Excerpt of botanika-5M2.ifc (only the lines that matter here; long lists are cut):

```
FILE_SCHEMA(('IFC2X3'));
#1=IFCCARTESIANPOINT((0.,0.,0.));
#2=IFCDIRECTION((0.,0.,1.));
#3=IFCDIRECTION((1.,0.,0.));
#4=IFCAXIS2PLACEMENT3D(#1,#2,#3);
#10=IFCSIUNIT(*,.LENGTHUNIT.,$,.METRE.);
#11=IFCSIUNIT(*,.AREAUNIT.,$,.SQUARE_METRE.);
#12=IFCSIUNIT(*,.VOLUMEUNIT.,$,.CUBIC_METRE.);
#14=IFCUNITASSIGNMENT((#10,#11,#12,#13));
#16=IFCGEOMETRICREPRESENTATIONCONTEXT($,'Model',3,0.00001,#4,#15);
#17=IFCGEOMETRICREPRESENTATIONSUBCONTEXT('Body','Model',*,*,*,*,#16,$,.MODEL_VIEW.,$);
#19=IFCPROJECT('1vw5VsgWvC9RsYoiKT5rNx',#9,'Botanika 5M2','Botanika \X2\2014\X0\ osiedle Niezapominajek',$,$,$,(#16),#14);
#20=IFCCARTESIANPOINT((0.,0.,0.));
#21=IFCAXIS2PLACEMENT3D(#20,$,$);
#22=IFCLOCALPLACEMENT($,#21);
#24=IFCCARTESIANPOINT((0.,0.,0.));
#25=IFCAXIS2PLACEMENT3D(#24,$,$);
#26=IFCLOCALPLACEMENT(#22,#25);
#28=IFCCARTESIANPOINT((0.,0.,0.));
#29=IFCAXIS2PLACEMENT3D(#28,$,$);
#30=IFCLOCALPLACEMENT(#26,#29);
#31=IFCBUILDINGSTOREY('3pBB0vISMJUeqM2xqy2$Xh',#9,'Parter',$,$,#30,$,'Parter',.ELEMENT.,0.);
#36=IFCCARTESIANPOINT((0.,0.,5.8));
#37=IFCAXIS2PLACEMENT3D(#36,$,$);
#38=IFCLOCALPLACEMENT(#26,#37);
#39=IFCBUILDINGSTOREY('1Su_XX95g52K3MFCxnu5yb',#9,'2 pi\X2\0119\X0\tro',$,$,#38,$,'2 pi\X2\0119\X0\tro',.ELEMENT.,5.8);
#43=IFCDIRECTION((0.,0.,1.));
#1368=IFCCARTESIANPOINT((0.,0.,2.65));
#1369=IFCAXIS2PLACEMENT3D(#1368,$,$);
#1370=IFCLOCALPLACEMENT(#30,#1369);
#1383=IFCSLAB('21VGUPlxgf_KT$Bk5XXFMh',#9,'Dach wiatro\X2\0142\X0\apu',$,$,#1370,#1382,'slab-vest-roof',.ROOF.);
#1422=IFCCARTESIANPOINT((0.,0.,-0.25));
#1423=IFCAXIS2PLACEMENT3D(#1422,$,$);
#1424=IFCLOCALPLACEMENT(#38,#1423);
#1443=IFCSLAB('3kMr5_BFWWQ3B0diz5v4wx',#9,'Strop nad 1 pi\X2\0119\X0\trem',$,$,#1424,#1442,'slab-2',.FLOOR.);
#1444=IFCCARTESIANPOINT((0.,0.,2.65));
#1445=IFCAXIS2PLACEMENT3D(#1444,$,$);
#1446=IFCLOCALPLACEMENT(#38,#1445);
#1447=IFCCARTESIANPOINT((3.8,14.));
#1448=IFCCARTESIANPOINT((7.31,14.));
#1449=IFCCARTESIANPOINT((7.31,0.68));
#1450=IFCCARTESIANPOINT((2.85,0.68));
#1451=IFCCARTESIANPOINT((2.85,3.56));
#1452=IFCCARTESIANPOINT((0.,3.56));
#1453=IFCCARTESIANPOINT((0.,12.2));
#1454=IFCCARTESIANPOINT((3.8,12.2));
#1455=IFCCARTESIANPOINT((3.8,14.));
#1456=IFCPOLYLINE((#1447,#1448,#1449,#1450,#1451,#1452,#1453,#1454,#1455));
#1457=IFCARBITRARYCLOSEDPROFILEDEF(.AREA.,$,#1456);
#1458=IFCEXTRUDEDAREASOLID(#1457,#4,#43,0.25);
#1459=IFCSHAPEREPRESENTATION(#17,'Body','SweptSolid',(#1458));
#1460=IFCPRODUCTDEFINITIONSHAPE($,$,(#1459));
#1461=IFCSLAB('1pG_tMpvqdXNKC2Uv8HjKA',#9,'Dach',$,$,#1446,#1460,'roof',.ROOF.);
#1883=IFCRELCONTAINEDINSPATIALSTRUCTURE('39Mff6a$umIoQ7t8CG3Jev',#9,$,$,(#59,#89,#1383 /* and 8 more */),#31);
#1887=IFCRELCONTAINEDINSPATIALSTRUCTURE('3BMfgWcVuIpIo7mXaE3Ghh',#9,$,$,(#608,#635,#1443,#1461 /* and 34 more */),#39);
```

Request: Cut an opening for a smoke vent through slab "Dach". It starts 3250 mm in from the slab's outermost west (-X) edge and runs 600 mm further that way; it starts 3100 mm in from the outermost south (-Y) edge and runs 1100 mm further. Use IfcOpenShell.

```python
import numpy as np
import ifcopenshell
import ifcopenshell.api.feature
import ifcopenshell.api.geometry
import ifcopenshell.api.root
import ifcopenshell.geom
import ifcopenshell.util.placement
import ifcopenshell.util.representation
import ifcopenshell.util.shape
import ifcopenshell.util.unit

model = ifcopenshell.open("botanika-5M2.ifc")
unit_scale = ifcopenshell.util.unit.calculate_unit_scale(model)
settings = ifcopenshell.geom.settings()


def volume(element):
    """Net volume in cubic metres, openings subtracted."""
    shape = ifcopenshell.geom.create_shape(settings, element)
    return ifcopenshell.util.shape.get_volume(shape.geometry)


slab = model.by_guid("1pG_tMpvqdXNKC2Uv8HjKA")
before = volume(slab)

# Extent in the slab's own axes, in metres. The edges named are its -X and -Y sides.
slab_shape = ifcopenshell.geom.create_shape(settings, slab)
vertices = ifcopenshell.util.shape.get_vertices(slab_shape.geometry)
x_min, y_min, bottom = vertices.min(axis=0)
top = vertices[:, 2].max()

opening = ifcopenshell.api.root.create_entity(model, ifc_class="IfcOpeningElement", name="Smoke vent opening")
context = ifcopenshell.util.representation.get_context(model, "Model", "Body", "MODEL_VIEW")
width, depth = 0.6, 1.1
outline = [(0.0, 0.0), (width, 0.0), (width, depth), (0.0, depth), (0.0, 0.0)]
# Overshoot both faces by 50 mm so the cut is clean.
shape = ifcopenshell.api.geometry.add_slab_representation(
    model, context=context, depth=top - bottom + 0.1, polyline=outline
)
ifcopenshell.api.geometry.assign_representation(model, product=opening, representation=shape)

matrix = ifcopenshell.util.placement.get_local_placement(slab.ObjectPlacement)
matrix[:, 3] = matrix @ np.append(np.array([x_min + 3.25, y_min + 3.1, bottom - 0.05]) / unit_scale, 1.0)
ifcopenshell.api.geometry.edit_object_placement(model, product=opening, matrix=matrix, is_si=False)
ifcopenshell.api.feature.add_feature(model, feature=opening, element=slab)

after = volume(slab)

print(f"slab volume {before:.3f} -> {after:.3f} m3")

model.write("botanika-5M2_v2.ifc")
```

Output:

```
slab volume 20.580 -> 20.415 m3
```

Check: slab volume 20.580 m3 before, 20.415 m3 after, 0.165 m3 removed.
